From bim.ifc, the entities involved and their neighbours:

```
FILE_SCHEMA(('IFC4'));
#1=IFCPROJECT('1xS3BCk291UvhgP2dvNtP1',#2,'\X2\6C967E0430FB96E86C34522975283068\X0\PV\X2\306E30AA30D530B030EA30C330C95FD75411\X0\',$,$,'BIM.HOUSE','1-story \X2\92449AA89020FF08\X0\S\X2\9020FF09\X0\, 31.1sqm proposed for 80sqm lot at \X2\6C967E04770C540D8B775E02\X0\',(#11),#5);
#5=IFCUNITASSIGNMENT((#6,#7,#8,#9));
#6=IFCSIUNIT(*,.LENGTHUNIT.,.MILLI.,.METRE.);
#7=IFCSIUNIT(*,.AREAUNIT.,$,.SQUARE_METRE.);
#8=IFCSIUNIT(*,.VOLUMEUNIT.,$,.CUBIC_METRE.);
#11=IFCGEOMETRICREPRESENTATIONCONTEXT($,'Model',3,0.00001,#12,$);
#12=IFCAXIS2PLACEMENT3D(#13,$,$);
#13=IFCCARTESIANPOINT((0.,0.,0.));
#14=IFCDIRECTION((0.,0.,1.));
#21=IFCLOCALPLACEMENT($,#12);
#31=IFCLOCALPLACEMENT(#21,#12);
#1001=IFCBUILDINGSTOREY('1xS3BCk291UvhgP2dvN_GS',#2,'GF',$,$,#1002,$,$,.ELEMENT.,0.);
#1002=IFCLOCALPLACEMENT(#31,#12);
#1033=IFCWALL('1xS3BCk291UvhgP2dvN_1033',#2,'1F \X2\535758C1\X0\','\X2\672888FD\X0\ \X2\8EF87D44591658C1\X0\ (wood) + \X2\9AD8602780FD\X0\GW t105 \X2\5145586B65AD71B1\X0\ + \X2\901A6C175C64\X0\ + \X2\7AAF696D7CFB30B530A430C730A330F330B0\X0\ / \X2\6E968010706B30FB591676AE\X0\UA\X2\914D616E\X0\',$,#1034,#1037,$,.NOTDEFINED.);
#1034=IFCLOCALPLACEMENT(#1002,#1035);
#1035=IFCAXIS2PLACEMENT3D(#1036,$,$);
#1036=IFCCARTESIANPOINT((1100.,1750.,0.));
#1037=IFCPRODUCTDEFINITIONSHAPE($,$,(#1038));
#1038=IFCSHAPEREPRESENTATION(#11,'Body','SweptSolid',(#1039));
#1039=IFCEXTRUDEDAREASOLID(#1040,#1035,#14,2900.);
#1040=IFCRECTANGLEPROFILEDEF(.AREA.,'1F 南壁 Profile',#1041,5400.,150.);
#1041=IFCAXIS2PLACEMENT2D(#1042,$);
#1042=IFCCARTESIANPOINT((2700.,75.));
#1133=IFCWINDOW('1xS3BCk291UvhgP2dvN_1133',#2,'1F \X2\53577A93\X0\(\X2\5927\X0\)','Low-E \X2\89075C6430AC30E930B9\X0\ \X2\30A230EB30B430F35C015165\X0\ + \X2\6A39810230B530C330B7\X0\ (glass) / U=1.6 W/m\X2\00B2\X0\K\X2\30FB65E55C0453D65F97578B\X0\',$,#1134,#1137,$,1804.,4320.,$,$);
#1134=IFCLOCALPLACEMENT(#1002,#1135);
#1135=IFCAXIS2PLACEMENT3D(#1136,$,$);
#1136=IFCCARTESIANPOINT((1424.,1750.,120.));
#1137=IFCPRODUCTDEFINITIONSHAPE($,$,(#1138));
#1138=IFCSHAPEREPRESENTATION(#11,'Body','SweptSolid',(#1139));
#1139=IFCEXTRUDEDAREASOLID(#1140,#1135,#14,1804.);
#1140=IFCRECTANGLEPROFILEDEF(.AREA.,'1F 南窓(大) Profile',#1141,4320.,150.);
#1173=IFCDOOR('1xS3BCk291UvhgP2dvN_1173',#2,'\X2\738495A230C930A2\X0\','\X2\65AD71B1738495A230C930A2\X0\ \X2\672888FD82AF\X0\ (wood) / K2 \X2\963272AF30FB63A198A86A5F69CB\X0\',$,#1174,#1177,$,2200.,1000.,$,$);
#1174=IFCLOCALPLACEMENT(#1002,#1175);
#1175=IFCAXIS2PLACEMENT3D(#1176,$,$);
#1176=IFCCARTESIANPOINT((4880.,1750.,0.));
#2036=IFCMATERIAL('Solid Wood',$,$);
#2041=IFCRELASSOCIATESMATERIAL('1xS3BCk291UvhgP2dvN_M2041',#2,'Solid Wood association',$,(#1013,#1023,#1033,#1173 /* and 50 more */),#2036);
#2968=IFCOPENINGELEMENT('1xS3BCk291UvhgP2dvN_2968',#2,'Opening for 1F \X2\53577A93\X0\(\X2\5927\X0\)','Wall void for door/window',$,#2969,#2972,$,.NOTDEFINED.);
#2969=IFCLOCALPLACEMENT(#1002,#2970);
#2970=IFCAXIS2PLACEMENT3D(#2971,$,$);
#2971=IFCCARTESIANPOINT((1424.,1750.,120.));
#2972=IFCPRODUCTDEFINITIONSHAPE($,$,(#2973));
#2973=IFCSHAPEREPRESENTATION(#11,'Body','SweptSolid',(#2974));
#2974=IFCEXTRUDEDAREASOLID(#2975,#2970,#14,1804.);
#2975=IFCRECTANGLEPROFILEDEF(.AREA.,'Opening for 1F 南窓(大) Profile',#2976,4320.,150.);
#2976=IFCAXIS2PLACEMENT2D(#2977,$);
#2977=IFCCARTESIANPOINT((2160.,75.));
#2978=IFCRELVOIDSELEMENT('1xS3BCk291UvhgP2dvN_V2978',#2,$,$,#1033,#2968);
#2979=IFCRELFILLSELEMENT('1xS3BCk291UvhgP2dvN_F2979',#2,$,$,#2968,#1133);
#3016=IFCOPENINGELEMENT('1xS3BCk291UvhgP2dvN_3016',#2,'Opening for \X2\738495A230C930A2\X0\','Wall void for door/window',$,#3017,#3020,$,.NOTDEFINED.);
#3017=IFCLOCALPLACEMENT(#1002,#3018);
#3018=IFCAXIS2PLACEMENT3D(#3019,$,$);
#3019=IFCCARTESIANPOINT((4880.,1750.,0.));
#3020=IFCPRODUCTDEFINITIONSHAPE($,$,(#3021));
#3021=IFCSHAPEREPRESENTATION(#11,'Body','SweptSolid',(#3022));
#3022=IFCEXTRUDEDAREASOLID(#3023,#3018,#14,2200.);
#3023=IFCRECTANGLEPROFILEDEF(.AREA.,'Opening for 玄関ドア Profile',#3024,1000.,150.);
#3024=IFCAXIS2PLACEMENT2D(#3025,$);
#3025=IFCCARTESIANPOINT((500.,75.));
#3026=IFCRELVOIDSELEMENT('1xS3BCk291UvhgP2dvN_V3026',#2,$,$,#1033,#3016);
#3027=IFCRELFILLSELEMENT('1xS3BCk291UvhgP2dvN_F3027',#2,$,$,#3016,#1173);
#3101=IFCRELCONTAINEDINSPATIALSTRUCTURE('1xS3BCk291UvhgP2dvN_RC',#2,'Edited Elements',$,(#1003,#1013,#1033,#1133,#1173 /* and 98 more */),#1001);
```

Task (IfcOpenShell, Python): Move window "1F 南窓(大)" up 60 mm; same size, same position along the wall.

```python
import numpy as np
import ifcopenshell
import ifcopenshell.api.geometry
import ifcopenshell.util.placement
import ifcopenshell.util.unit

model = ifcopenshell.open("bim.ifc")
unit_scale = ifcopenshell.util.unit.calculate_unit_scale(model)

window = model.by_guid("1xS3BCk291UvhgP2dvN_1133")
opening = window.FillsVoids[0].RelatingOpeningElement
dz = 60.0

shift = np.array([0.0, 0.0, dz])
# The window is not placed relative to its opening, so move both.
for product in (opening, window):
    matrix = ifcopenshell.util.placement.get_local_placement(product.ObjectPlacement)
    matrix[:3, 3] += shift
    ifcopenshell.api.geometry.edit_object_placement(model, product=product, matrix=matrix, is_si=False)

print(f"moved by {dz * unit_scale:+.3f} m")

model.write("bim-out.ifc")
```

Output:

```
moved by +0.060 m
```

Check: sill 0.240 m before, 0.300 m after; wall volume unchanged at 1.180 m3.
